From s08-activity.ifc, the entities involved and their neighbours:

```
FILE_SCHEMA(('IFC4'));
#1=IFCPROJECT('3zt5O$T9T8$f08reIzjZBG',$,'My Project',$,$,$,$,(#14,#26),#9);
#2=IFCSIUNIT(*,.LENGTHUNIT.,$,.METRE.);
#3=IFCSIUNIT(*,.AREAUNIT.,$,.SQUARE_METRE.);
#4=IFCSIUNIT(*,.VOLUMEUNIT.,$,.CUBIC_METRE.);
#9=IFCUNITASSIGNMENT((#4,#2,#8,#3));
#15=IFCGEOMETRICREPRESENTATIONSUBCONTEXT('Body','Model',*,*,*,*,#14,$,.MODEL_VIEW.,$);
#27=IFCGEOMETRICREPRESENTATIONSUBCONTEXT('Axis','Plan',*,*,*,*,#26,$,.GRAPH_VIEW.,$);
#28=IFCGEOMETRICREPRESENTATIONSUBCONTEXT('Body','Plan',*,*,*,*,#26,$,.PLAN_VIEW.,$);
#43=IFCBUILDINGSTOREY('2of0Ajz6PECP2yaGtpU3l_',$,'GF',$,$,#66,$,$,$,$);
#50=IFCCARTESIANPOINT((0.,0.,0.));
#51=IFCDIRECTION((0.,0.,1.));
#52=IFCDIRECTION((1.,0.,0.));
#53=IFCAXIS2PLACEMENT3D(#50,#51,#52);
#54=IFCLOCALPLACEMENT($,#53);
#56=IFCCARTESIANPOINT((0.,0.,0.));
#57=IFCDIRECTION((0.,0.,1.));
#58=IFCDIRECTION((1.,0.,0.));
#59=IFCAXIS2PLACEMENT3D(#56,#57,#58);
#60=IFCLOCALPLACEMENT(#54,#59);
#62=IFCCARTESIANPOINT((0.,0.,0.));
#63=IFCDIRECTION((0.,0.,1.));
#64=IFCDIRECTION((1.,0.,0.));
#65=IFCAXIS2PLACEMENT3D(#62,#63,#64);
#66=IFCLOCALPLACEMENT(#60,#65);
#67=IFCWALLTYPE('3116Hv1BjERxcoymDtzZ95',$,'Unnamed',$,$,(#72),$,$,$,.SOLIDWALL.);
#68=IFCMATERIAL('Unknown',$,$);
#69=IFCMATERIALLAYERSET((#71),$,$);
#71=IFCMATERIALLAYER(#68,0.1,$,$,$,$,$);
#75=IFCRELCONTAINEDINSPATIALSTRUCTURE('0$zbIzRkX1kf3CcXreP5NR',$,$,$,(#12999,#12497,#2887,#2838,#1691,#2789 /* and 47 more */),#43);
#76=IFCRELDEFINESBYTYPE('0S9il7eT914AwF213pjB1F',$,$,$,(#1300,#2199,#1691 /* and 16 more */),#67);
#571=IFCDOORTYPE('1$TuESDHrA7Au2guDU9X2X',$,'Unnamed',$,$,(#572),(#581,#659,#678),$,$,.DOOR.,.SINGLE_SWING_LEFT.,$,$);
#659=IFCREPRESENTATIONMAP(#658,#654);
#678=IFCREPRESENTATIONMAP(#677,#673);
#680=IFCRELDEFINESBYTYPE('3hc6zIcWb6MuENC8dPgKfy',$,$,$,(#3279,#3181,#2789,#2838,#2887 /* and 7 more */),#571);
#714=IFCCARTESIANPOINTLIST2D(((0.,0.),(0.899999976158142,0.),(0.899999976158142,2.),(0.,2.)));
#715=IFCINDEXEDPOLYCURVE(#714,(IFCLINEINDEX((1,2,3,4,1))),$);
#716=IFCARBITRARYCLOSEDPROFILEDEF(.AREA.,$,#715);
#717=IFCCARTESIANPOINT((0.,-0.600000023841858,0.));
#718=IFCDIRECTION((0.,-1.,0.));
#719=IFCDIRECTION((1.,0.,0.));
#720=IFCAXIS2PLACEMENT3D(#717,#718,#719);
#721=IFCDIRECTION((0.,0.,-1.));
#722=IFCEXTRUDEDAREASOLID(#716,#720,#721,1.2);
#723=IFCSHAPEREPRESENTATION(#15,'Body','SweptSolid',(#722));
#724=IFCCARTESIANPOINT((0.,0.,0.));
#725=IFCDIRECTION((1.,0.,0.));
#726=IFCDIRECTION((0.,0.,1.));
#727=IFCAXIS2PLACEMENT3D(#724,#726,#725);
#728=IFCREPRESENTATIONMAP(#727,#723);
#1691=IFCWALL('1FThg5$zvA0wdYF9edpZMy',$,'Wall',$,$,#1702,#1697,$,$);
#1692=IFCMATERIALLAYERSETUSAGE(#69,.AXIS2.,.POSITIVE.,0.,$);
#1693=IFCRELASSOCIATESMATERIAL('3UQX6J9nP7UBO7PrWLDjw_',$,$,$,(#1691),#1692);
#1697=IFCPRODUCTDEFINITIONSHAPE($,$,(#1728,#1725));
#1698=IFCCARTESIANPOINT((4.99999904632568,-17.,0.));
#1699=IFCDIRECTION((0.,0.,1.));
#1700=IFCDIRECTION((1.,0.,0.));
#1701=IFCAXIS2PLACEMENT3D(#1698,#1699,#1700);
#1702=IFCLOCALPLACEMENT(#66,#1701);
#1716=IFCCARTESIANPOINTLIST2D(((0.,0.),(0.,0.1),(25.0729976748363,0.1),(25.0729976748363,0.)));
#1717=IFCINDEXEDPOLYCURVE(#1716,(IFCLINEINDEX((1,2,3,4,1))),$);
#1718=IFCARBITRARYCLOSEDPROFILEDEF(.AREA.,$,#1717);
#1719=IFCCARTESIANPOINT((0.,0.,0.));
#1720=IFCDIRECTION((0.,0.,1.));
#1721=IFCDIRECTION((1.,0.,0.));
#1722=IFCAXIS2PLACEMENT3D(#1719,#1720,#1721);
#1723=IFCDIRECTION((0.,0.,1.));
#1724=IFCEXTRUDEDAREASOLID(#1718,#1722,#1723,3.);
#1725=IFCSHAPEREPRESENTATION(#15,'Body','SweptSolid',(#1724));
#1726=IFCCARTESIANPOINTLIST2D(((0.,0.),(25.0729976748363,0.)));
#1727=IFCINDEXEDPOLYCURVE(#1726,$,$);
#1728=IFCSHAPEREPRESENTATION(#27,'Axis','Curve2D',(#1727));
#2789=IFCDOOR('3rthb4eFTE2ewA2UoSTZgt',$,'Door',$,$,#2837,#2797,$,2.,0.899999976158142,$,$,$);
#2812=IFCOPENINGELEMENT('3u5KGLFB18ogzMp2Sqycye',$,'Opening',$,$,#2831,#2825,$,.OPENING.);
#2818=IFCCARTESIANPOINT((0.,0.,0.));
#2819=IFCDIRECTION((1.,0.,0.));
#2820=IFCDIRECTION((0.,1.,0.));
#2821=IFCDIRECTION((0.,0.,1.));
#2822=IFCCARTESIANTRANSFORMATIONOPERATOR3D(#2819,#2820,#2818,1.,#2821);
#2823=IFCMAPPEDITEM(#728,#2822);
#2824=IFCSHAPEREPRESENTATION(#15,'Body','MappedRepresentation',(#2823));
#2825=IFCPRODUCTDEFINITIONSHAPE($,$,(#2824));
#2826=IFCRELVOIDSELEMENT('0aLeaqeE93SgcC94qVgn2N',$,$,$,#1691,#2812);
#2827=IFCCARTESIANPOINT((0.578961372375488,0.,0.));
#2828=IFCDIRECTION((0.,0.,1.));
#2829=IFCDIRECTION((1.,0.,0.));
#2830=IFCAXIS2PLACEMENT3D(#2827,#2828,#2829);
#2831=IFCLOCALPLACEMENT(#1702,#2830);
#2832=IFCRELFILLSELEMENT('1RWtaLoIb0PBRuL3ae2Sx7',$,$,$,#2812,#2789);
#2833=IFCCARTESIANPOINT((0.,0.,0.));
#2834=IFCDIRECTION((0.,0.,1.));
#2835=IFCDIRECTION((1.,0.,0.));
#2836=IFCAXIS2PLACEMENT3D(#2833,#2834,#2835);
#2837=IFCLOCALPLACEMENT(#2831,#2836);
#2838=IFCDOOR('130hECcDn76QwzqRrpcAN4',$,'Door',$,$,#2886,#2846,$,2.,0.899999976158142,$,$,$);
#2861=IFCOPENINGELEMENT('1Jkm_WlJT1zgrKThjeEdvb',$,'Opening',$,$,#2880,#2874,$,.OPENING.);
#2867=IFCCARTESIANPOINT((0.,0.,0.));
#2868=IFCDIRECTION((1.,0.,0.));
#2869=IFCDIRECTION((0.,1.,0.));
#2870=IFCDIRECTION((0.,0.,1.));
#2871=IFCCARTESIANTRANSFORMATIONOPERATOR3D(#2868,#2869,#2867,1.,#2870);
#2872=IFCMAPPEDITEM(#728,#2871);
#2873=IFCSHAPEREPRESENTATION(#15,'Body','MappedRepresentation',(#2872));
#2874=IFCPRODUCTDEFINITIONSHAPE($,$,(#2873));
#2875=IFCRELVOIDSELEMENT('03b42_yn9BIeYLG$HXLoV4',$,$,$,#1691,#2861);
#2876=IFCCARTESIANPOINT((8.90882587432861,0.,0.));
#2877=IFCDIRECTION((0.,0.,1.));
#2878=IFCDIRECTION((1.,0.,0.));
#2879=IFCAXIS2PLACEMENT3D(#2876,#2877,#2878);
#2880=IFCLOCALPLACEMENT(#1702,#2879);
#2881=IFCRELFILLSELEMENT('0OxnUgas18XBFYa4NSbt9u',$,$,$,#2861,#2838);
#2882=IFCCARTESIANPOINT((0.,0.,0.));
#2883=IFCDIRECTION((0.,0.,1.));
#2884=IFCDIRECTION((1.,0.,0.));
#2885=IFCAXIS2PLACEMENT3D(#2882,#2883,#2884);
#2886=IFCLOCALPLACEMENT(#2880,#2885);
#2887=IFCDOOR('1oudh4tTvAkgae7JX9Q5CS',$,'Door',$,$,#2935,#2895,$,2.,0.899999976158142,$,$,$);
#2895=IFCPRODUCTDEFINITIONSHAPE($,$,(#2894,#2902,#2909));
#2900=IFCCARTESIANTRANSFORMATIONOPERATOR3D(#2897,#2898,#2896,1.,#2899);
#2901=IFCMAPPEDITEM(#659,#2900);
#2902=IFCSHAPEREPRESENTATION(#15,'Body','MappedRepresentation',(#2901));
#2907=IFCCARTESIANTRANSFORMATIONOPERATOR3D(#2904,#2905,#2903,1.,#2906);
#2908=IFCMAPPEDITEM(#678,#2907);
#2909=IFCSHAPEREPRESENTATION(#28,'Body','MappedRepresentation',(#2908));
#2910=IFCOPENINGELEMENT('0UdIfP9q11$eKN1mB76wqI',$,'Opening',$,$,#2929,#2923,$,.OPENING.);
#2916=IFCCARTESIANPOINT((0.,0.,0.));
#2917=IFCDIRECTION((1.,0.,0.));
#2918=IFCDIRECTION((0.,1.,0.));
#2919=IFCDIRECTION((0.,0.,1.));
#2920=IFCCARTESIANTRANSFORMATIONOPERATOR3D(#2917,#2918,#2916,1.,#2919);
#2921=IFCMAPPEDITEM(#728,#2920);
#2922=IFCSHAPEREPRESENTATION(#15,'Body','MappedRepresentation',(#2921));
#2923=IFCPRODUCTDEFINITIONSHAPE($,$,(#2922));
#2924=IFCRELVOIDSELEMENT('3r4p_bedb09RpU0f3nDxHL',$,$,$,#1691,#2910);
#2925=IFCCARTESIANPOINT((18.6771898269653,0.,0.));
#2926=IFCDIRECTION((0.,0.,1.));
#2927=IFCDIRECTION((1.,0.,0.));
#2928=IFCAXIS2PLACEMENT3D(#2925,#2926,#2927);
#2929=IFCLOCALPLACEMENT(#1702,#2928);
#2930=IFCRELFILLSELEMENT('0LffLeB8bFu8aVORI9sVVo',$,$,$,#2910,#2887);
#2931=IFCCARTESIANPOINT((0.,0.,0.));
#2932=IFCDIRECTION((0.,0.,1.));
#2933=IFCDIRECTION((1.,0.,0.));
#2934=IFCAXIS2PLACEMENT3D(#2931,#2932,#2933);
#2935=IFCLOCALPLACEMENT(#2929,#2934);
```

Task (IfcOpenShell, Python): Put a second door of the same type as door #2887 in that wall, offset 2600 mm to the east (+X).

```python
import ifcopenshell
import ifcopenshell.api.feature
import ifcopenshell.api.geometry
import ifcopenshell.api.root
import ifcopenshell.geom
import ifcopenshell.util.element
import ifcopenshell.util.placement
import ifcopenshell.util.shape
import ifcopenshell.util.unit

model = ifcopenshell.open("s08-activity.ifc")
unit_scale = ifcopenshell.util.unit.calculate_unit_scale(model)
settings = ifcopenshell.geom.settings()


def volume(element):
    """Net volume in cubic metres, openings subtracted."""
    shape = ifcopenshell.geom.create_shape(settings, element)
    return ifcopenshell.util.shape.get_volume(shape.geometry)


door = model.by_id(2887)
opening = door.FillsVoids[0].RelatingOpeningElement
wall = opening.VoidsElements[0].RelatingBuildingElement
before = volume(wall)
shift = ifcopenshell.util.placement.get_local_placement(wall.ObjectPlacement)[:3, 0] * 2.6 / unit_scale

# copy_class copies the void relationship, type, container and properties, but no geometry.
new_opening = ifcopenshell.api.root.copy_class(model, product=opening)
new_opening.Representation = ifcopenshell.util.element.copy_deep(
    model, opening.Representation, exclude=["IfcGeometricRepresentationContext", "IfcRepresentationMap"]
)
new_door = ifcopenshell.api.root.copy_class(model, product=door)
new_door.Representation = ifcopenshell.util.element.copy_deep(
    model, door.Representation, exclude=["IfcGeometricRepresentationContext", "IfcRepresentationMap"]
)
ifcopenshell.api.feature.add_filling(model, opening=new_opening, element=new_door)

for old, new in ((opening, new_opening), (door, new_door)):
    matrix = ifcopenshell.util.placement.get_local_placement(old.ObjectPlacement)
    matrix[:3, 3] += shift
    ifcopenshell.api.geometry.edit_object_placement(model, product=new, matrix=matrix, is_si=False)

after = volume(wall)

print(f"wall volume {before:.3f} -> {after:.3f} m3")

model.write("s08-activity_edited.ifc")
```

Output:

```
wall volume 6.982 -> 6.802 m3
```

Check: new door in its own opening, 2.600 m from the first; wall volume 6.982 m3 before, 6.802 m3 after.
